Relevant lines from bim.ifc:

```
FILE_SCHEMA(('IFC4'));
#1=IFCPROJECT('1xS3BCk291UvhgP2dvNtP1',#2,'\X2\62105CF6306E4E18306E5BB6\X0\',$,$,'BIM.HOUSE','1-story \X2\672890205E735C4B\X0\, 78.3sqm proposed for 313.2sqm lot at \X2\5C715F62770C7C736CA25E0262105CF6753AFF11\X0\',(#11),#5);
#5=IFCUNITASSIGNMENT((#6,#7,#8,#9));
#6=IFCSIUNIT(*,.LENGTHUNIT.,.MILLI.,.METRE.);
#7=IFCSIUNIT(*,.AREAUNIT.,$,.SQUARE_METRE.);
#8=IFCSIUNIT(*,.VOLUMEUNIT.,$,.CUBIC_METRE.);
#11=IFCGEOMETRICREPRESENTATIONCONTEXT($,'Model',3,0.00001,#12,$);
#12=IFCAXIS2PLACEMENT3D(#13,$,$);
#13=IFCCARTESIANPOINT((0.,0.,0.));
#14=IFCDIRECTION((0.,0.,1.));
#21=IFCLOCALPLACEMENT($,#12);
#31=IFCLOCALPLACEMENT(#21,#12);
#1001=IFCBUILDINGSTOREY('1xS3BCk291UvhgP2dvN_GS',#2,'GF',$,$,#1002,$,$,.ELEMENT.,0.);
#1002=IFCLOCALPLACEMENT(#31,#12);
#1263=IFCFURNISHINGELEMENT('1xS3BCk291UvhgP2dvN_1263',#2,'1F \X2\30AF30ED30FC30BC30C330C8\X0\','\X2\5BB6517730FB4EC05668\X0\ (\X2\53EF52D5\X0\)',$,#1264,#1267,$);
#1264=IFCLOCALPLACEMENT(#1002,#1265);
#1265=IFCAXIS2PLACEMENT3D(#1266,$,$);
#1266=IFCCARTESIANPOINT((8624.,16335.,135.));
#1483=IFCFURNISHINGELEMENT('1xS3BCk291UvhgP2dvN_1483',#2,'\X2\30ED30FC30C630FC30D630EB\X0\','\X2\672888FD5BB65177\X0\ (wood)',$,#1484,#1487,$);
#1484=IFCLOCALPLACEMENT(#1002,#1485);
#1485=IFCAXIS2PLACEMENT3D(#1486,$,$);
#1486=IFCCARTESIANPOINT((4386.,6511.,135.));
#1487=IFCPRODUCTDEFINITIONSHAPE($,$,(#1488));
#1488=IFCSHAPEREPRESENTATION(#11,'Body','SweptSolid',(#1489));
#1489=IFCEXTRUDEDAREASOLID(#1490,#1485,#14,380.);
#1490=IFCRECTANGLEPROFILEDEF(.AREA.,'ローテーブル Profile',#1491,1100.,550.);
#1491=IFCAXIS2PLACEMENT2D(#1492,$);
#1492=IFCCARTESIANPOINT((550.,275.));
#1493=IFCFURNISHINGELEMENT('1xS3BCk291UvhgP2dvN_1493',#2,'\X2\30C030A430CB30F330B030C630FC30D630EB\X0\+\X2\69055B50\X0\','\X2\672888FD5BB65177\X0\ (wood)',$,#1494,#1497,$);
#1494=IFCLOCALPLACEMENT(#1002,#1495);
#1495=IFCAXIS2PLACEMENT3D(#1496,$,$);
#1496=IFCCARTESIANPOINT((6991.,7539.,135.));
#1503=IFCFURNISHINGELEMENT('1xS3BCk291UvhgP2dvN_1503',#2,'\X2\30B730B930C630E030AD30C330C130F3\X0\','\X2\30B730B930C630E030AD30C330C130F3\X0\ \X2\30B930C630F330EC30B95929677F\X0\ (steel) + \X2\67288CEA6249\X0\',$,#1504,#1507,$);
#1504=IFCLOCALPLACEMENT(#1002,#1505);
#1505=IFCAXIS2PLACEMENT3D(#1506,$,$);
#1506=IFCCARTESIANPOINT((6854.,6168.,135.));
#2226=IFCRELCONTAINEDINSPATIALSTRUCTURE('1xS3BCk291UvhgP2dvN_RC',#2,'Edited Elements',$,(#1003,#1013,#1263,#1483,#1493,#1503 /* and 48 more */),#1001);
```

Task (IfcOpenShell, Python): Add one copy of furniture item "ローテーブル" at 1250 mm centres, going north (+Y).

```python
import numpy as np
import ifcopenshell
import ifcopenshell.api.geometry
import ifcopenshell.api.root
import ifcopenshell.util.element
import ifcopenshell.util.placement
import ifcopenshell.util.unit

model = ifcopenshell.open("bim.ifc")
unit_scale = ifcopenshell.util.unit.calculate_unit_scale(model)


def reuse_history(source, copy):
    """copy_class also copies each property set's owner history, people and application; keep the originals."""
    for rel in copy.IsDefinedBy:
        if rel.is_a("IfcRelDefinesByProperties") and (history := rel.RelatingPropertyDefinition.OwnerHistory):
            rel.RelatingPropertyDefinition.OwnerHistory = source.OwnerHistory
            ifcopenshell.util.element.remove_deep2(model, history)


source = model.by_id(1483)
base = ifcopenshell.util.placement.get_local_placement(source.ObjectPlacement)
step = np.array([0.0, 1.0, 0.0]) * 1.25 / unit_scale

for i in range(1, 2):
    copy = ifcopenshell.api.root.copy_class(model, product=source)
    copy.Representation = ifcopenshell.util.element.copy_deep(
        model, source.Representation, exclude=["IfcGeometricRepresentationContext", "IfcRepresentationMap"]
    )
    reuse_history(source, copy)
    matrix = base.copy()
    matrix[:3, 3] += i * step
    print("added at", matrix[:3, 3].round(3) + 0.0)
    ifcopenshell.api.geometry.edit_object_placement(model, product=copy, matrix=matrix, is_si=False)

model.write("bim_rev.ifc")
```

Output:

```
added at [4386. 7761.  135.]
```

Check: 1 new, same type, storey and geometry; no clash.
